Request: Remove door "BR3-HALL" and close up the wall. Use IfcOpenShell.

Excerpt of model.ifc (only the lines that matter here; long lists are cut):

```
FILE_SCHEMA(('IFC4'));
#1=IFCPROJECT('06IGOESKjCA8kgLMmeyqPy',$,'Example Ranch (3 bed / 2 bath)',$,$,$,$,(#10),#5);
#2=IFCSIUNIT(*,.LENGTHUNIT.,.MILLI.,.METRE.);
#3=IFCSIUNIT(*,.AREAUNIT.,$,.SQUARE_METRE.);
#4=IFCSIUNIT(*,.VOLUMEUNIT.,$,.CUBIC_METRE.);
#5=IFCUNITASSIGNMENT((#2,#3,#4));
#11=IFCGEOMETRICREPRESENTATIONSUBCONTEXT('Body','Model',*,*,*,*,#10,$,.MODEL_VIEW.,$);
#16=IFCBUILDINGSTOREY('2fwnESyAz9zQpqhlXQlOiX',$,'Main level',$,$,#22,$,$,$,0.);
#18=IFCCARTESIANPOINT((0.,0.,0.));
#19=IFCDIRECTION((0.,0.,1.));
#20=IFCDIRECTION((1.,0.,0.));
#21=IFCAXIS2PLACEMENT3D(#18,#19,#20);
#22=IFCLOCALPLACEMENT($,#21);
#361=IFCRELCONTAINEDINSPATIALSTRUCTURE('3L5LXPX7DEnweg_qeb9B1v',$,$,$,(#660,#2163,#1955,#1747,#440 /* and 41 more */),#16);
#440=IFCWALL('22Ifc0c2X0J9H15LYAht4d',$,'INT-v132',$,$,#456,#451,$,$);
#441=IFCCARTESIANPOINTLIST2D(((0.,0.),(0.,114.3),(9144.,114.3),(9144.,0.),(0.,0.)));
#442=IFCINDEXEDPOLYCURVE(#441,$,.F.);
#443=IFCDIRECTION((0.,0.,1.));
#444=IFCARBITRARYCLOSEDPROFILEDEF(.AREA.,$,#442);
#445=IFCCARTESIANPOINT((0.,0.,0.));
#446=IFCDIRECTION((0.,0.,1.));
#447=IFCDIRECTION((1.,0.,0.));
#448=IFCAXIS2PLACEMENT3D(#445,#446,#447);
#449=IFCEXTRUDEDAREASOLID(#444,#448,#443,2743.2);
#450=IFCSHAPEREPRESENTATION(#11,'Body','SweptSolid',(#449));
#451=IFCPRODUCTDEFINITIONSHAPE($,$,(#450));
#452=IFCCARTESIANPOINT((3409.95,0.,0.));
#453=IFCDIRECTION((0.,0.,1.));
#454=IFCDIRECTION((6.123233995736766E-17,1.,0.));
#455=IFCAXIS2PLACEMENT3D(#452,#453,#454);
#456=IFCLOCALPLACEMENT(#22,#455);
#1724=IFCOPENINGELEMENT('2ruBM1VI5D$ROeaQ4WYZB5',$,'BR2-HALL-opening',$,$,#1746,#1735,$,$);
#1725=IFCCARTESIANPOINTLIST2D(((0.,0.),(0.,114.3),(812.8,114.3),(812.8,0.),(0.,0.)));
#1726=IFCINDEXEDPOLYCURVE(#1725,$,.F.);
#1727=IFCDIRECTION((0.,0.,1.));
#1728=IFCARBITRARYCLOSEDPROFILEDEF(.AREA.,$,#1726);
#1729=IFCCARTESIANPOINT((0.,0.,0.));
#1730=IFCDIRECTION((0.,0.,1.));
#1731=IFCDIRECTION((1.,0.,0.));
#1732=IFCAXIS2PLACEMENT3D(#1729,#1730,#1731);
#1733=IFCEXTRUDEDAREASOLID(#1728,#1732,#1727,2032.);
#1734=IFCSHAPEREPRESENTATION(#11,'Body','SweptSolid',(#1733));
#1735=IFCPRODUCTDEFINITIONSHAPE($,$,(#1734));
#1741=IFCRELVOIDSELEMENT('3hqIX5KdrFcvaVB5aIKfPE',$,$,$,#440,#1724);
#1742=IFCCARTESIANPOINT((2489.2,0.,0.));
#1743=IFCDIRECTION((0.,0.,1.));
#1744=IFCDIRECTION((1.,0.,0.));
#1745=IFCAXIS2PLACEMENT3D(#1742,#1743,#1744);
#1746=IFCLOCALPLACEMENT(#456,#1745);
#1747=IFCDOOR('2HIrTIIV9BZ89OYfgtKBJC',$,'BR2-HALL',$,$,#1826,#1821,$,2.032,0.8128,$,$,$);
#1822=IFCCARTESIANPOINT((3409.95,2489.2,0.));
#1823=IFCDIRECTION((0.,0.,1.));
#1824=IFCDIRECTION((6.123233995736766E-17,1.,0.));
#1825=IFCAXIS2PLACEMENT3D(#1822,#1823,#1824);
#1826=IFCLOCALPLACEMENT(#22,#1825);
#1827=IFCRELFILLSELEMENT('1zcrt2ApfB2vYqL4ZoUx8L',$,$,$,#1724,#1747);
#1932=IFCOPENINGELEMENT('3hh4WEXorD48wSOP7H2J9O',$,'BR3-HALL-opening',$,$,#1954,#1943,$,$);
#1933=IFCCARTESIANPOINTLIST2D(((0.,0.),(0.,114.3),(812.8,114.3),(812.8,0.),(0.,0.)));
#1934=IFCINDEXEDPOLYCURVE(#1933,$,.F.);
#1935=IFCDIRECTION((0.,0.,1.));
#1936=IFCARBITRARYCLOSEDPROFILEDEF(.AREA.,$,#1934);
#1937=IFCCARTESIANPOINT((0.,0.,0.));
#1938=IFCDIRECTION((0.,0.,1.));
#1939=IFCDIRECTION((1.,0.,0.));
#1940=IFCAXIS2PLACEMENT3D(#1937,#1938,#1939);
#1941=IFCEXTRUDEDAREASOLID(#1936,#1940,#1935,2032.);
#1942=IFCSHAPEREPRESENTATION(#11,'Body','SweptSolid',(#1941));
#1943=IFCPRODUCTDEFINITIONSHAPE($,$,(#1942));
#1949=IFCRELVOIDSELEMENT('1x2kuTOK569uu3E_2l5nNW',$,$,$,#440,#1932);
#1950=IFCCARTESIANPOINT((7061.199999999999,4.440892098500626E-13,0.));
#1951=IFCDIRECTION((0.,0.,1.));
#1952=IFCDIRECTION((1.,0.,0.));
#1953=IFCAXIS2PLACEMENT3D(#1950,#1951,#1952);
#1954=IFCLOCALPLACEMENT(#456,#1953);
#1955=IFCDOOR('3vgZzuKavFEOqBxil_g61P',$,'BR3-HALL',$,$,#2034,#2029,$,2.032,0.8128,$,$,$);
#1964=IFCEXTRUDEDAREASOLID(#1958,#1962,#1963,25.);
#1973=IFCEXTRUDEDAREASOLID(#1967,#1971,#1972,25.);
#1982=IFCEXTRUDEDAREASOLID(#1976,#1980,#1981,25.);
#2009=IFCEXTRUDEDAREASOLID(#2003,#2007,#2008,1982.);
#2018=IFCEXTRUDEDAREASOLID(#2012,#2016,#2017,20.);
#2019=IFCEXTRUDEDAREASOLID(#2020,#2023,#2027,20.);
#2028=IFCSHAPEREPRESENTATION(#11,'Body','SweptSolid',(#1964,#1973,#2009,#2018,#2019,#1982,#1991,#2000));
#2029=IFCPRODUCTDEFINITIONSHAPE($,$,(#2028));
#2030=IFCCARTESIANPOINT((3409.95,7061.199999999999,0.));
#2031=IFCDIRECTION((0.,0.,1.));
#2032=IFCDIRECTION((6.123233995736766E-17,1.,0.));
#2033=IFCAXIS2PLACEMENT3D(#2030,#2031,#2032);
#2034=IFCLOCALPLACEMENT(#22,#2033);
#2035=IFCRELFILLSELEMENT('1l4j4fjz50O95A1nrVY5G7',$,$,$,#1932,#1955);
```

```python
import ifcopenshell
import ifcopenshell.api.feature
import ifcopenshell.api.root
import ifcopenshell.geom
import ifcopenshell.util.shape

model = ifcopenshell.open("model.ifc")
settings = ifcopenshell.geom.settings()


def volume(element):
    """Net volume in cubic metres, openings subtracted."""
    shape = ifcopenshell.geom.create_shape(settings, element)
    return ifcopenshell.util.shape.get_volume(shape.geometry)


door = model.by_guid("3vgZzuKavFEOqBxil_g61P")
opening = door.FillsVoids[0].RelatingOpeningElement
wall = opening.VoidsElements[0].RelatingBuildingElement
before = volume(wall)

ifcopenshell.api.root.remove_product(model, product=door)
ifcopenshell.api.feature.remove_feature(model, feature=opening)

after = volume(wall)

print(f"wall volume {before:.3f} -> {after:.3f} m3")

model.write("model_v2.ifc")
```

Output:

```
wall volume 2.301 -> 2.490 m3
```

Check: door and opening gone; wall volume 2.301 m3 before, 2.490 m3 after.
